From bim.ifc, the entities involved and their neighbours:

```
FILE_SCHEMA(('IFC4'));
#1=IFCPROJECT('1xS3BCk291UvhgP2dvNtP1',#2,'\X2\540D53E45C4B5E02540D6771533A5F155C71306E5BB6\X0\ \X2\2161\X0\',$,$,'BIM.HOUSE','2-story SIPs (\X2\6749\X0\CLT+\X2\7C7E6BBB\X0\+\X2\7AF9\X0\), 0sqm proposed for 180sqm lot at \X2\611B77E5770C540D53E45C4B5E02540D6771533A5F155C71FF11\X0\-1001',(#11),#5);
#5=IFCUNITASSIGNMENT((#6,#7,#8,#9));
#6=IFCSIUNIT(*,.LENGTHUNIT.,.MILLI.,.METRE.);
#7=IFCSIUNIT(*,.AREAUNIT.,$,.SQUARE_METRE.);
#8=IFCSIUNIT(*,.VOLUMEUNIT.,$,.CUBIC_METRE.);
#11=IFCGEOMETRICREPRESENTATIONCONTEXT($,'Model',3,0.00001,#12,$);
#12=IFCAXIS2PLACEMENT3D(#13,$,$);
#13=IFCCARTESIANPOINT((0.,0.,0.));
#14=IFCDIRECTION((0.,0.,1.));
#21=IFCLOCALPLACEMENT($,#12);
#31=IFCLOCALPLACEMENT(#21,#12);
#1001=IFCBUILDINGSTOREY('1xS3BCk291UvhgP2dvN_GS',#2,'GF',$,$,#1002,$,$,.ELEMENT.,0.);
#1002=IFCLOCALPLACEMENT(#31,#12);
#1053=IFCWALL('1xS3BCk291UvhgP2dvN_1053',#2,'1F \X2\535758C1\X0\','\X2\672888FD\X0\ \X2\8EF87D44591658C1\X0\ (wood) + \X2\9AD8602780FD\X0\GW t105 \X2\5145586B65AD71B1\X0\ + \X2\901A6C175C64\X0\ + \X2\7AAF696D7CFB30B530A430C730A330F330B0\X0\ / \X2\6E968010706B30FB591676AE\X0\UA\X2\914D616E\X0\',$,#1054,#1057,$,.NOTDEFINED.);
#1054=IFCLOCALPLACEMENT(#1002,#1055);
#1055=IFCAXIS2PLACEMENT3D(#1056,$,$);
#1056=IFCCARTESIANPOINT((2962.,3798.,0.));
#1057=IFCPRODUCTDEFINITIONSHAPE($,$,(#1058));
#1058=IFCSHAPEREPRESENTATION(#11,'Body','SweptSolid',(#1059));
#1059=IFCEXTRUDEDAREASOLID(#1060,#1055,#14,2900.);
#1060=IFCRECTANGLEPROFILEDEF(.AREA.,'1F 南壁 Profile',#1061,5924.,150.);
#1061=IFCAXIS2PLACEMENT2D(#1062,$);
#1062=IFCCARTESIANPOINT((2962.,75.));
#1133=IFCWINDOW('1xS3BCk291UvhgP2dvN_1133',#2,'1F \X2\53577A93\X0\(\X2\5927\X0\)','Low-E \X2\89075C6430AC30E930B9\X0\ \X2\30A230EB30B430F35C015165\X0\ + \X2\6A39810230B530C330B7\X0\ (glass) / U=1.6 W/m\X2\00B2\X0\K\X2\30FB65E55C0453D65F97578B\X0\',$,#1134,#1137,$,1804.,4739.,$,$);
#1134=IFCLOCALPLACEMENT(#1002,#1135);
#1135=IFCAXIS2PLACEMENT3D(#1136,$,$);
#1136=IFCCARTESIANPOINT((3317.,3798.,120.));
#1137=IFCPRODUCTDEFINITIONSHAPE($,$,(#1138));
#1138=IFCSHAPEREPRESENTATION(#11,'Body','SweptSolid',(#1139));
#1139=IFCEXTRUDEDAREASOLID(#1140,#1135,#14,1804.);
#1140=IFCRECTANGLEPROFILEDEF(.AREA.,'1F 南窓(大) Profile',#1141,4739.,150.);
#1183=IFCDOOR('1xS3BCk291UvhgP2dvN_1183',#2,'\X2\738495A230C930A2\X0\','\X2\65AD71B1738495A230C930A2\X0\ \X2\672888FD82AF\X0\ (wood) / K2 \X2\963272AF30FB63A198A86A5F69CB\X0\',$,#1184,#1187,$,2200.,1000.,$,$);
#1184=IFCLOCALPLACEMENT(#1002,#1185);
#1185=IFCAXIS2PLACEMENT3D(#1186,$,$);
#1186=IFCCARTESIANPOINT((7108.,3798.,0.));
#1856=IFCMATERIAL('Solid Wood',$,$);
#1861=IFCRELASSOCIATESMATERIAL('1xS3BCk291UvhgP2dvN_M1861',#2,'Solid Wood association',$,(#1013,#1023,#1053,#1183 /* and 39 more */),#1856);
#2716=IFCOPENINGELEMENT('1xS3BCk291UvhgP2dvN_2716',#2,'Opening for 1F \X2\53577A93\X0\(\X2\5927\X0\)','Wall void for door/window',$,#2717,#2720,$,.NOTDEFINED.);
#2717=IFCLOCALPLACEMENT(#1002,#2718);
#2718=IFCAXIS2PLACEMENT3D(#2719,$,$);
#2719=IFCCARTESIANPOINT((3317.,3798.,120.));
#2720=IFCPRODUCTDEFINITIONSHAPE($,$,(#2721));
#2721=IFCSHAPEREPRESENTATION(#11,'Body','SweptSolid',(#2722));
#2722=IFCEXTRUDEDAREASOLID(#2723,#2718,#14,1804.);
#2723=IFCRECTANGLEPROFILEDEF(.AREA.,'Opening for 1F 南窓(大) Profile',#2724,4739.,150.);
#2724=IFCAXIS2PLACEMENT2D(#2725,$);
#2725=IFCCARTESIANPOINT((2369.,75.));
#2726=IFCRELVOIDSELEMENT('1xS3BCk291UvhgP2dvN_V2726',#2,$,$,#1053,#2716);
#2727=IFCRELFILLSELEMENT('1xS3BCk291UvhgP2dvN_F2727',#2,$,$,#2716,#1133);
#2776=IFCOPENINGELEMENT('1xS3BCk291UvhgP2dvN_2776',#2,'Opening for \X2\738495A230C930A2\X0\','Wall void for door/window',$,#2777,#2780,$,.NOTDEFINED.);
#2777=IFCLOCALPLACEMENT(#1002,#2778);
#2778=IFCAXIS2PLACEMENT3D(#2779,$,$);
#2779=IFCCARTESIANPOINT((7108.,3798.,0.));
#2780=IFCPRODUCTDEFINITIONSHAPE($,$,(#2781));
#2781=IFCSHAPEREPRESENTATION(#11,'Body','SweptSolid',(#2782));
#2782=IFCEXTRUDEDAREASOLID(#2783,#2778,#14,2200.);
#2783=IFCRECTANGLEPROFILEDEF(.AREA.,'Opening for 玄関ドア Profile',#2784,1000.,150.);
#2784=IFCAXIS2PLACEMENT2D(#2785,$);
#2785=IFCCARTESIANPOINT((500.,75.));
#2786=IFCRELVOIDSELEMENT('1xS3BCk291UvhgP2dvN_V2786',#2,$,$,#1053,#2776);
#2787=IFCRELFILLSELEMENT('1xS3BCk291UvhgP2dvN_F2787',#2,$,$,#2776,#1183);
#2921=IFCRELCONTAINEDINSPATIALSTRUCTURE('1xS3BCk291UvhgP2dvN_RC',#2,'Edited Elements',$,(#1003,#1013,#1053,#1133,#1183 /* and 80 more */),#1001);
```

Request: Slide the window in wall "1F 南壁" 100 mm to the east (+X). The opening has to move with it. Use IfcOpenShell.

```python
import ifcopenshell
import ifcopenshell.api.geometry
import ifcopenshell.util.placement
import ifcopenshell.util.unit

model = ifcopenshell.open("bim.ifc")
unit_scale = ifcopenshell.util.unit.calculate_unit_scale(model)

window = model.by_guid("1xS3BCk291UvhgP2dvN_1133")
opening = window.FillsVoids[0].RelatingOpeningElement
wall = opening.VoidsElements[0].RelatingBuildingElement

wall_matrix = ifcopenshell.util.placement.get_local_placement(wall.ObjectPlacement)
shift = wall_matrix[:3, 0] * 0.1 / unit_scale
before = ifcopenshell.util.placement.get_local_placement(window.ObjectPlacement)[:3, 3].copy()

# The window is not placed relative to its opening, so move both.
for product in (opening, window):
    matrix = ifcopenshell.util.placement.get_local_placement(product.ObjectPlacement)
    matrix[:3, 3] += shift
    ifcopenshell.api.geometry.edit_object_placement(model, product=product, matrix=matrix, is_si=False)

after = ifcopenshell.util.placement.get_local_placement(window.ObjectPlacement)[:3, 3]
print("window moved by", (after - before).round(3) + 0.0)

model.write("bim_edited.ifc")
```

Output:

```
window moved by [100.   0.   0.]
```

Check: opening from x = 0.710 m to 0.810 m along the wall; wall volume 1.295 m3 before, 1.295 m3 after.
